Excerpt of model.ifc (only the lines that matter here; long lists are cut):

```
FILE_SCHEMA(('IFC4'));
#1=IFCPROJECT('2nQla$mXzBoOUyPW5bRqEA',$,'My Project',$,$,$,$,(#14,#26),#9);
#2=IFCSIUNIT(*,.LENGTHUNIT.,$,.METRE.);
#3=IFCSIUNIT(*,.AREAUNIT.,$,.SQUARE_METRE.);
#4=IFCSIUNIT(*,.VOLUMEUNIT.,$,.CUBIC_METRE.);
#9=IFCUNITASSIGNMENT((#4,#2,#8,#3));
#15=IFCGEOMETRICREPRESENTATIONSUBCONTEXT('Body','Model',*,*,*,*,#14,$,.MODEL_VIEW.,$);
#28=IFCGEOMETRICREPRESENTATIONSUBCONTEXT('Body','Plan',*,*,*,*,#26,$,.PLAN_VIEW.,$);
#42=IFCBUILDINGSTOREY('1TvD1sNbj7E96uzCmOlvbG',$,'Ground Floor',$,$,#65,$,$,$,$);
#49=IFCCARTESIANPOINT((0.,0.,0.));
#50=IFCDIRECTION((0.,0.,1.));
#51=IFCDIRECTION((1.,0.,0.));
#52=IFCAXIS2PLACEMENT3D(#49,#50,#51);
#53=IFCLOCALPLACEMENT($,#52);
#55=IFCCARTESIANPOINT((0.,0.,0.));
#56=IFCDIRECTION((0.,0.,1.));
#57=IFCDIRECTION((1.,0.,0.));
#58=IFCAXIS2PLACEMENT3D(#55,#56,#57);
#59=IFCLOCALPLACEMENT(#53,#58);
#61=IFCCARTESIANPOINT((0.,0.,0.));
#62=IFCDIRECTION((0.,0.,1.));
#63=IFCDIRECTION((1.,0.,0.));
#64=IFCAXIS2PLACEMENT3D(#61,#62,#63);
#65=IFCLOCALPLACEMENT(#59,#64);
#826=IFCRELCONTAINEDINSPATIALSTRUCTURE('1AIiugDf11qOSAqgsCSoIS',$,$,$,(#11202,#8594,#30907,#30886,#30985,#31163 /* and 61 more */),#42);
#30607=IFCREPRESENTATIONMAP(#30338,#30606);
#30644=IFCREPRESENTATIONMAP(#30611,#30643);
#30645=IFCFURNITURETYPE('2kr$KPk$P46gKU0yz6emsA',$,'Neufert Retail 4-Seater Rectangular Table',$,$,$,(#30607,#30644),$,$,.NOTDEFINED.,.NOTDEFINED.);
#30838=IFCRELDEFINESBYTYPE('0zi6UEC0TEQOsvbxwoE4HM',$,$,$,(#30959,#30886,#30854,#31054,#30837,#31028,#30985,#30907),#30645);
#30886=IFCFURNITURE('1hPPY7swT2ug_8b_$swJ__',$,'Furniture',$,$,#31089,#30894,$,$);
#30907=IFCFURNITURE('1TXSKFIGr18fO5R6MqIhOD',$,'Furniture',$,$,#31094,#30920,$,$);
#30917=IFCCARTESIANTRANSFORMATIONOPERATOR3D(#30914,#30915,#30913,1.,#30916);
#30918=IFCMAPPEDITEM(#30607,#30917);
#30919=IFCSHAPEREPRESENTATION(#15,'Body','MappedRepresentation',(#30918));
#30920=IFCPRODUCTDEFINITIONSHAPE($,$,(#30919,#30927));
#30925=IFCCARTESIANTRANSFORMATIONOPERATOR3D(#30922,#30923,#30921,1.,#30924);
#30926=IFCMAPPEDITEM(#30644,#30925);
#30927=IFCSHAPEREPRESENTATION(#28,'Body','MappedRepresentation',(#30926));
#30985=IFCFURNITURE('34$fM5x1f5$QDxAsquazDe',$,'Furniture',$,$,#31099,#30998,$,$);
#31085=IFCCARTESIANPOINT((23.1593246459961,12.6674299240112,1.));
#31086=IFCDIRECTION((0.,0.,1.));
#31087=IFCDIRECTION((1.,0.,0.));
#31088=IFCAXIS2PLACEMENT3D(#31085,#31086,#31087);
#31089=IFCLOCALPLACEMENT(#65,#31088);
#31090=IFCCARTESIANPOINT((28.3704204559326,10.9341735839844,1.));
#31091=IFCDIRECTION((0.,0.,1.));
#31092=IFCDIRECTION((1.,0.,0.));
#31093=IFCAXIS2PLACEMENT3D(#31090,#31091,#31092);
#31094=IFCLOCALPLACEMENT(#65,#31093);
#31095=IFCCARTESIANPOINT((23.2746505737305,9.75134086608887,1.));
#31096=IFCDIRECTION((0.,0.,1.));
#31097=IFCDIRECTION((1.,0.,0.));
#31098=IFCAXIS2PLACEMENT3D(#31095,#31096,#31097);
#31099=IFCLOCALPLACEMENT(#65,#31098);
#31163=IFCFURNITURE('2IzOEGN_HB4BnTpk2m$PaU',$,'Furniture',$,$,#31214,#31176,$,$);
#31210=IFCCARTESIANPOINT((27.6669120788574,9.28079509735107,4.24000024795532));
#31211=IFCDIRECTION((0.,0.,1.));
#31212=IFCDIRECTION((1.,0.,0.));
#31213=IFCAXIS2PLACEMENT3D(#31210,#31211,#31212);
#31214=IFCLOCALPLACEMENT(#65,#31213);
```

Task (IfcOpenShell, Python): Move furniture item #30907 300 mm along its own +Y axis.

```python
import ifcopenshell
import ifcopenshell.api.geometry
import ifcopenshell.util.placement
import ifcopenshell.util.unit

model = ifcopenshell.open("model.ifc")
unit_scale = ifcopenshell.util.unit.calculate_unit_scale(model)

item = model.by_guid("1TXSKFIGr18fO5R6MqIhOD")
matrix = ifcopenshell.util.placement.get_local_placement(item.ObjectPlacement)
matrix[:3, 3] += matrix[:3, 1] * 0.3 / unit_scale
ifcopenshell.api.geometry.edit_object_placement(model, product=item, matrix=matrix, is_si=False)

print(ifcopenshell.util.placement.get_local_placement(item.ObjectPlacement).round(3) + 0.0)

model.write("model-out.ifc")
```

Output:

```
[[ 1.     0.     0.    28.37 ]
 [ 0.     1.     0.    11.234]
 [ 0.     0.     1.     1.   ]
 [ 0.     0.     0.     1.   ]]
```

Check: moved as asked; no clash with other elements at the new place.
